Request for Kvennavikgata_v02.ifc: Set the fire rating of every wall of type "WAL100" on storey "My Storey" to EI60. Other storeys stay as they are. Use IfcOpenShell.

First a look at what the model holds.

```python
import ifcopenshell
import ifcopenshell.util.element

model = ifcopenshell.open("Kvennavikgata_v02.ifc")
print(model.schema)
storey = next(s for s in model.by_type("IfcBuildingStorey") if s.Name == "My Storey")
walls = [e for e in ifcopenshell.util.element.get_decomposition(storey) if e.is_a("IfcWall")]
seen = {}
for e in walls:
    element_type = ifcopenshell.util.element.get_type(e)
    key = (element_type.Name if element_type != e and element_type else None, ifcopenshell.util.element.get_pset(e, "Pset_WallCommon", "FireRating"))
    seen[key] = seen.get(key, 0) + 1
for (name, value), count in sorted(seen.items(), key=str):
    print(count, "x", name, "|", value)
```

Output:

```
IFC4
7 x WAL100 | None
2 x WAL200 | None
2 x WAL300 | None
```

```python
import ifcopenshell
import ifcopenshell.api.pset
import ifcopenshell.util.element

model = ifcopenshell.open("Kvennavikgata_v02.ifc")

storey = next(s for s in model.by_type("IfcBuildingStorey") if s.Name == "My Storey")
walls = [e for e in ifcopenshell.util.element.get_decomposition(storey) if e.is_a("IfcWall")]

count = 0
for e in walls:
    element_type = ifcopenshell.util.element.get_type(e)
    if element_type in (None, e) or element_type.Name != "WAL100":
        continue
    # add_pset returns the element's existing set when there is one.
    pset = ifcopenshell.api.pset.add_pset(model, product=e, name="Pset_WallCommon")
    ifcopenshell.api.pset.edit_pset(model, pset=pset, properties={"FireRating": "EI60"})
    count += 1

print(count, "walls updated")

model.write("Kvennavikgata_v02_edited.ifc")
```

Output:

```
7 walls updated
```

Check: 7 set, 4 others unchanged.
